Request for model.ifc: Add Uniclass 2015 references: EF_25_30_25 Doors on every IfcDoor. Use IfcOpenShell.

First a look at what the model holds.

```python
import ifcopenshell

model = ifcopenshell.open("model.ifc")
print(model.schema)
print("classifications:", [c.Name for c in model.by_type("IfcClassification")])
for ifc_class in ("IfcDoor", "IfcRoof", "IfcStair", "IfcWall", "IfcWindow"):
    print(ifc_class, len(model.by_type(ifc_class)))
```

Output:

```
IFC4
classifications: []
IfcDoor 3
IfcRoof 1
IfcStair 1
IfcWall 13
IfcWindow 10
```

```python
import ifcopenshell
import ifcopenshell.api.classification

model = ifcopenshell.open("model.ifc")

system = ifcopenshell.api.classification.add_classification(model, classification="Uniclass 2015")

codes = {
    "IfcDoor": ("EF_25_30_25", "Doors"),
}
for ifc_class, (code, name) in codes.items():
    products = model.by_type(ifc_class)
    ifcopenshell.api.classification.add_reference(
        model, products=products, classification=system, identification=code, name=name
    )
    print(code, len(products))

model.write("model-out.ifc")
```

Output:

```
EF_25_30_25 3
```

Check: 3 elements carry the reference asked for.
